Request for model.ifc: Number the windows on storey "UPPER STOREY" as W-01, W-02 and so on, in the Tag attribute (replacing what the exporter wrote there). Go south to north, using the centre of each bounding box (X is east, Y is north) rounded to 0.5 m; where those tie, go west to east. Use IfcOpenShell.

First a look at what the model holds.

```python
import ifcopenshell
import ifcopenshell.util.element
import ifcopenshell.util.placement

model = ifcopenshell.open("model.ifc")
print(model.schema)
storey = next(s for s in model.by_type("IfcBuildingStorey") if s.Name == "UPPER STOREY")
windows = [e for e in ifcopenshell.util.element.get_decomposition(storey) if e.is_a("IfcWindow")]
for e in sorted(windows, key=lambda e: e.id()):
    origin = ifcopenshell.util.placement.get_local_placement(e.ObjectPlacement)[:3, 3]
    print(e.id(), e.Tag, e.Name, origin.round(2) + 0.0, sep=" | ")
```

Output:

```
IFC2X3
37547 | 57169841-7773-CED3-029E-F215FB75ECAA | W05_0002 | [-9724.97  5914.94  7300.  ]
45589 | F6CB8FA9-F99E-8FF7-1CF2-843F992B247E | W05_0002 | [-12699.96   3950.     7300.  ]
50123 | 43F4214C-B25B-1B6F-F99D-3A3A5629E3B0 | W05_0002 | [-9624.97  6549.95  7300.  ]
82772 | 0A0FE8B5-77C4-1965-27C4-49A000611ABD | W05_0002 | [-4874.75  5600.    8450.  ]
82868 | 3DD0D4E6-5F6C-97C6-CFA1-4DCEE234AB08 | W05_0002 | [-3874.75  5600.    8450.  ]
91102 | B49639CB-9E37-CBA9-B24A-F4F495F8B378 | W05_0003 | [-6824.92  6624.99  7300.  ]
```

```python
import ifcopenshell
import ifcopenshell.geom
import ifcopenshell.util.element
import ifcopenshell.util.shape

model = ifcopenshell.open("model.ifc")
settings = ifcopenshell.geom.settings()
settings.set("use-world-coords", True)


def centre(element):
    shape = ifcopenshell.geom.create_shape(settings, element)
    return ifcopenshell.util.shape.get_bbox_centroid(shape.geometry)


storey = next(s for s in model.by_type("IfcBuildingStorey") if s.Name == "UPPER STOREY")
windows = [e for e in ifcopenshell.util.element.get_decomposition(storey) if e.is_a("IfcWindow")]

# Insertion points can sit at a corner or the storey origin, so sort by the geometry (in metres).
centres = {e: centre(e) for e in windows}
windows.sort(key=lambda e: (round(centres[e][1] / 0.5), centres[e][0]))

for i, e in enumerate(windows, start=1):
    number = f"W-{i:02d}"
    e.Tag = number
    print(e.id(), number)

model.write("model-out.ifc")
```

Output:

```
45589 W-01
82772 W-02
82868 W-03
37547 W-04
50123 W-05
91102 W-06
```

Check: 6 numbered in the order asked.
